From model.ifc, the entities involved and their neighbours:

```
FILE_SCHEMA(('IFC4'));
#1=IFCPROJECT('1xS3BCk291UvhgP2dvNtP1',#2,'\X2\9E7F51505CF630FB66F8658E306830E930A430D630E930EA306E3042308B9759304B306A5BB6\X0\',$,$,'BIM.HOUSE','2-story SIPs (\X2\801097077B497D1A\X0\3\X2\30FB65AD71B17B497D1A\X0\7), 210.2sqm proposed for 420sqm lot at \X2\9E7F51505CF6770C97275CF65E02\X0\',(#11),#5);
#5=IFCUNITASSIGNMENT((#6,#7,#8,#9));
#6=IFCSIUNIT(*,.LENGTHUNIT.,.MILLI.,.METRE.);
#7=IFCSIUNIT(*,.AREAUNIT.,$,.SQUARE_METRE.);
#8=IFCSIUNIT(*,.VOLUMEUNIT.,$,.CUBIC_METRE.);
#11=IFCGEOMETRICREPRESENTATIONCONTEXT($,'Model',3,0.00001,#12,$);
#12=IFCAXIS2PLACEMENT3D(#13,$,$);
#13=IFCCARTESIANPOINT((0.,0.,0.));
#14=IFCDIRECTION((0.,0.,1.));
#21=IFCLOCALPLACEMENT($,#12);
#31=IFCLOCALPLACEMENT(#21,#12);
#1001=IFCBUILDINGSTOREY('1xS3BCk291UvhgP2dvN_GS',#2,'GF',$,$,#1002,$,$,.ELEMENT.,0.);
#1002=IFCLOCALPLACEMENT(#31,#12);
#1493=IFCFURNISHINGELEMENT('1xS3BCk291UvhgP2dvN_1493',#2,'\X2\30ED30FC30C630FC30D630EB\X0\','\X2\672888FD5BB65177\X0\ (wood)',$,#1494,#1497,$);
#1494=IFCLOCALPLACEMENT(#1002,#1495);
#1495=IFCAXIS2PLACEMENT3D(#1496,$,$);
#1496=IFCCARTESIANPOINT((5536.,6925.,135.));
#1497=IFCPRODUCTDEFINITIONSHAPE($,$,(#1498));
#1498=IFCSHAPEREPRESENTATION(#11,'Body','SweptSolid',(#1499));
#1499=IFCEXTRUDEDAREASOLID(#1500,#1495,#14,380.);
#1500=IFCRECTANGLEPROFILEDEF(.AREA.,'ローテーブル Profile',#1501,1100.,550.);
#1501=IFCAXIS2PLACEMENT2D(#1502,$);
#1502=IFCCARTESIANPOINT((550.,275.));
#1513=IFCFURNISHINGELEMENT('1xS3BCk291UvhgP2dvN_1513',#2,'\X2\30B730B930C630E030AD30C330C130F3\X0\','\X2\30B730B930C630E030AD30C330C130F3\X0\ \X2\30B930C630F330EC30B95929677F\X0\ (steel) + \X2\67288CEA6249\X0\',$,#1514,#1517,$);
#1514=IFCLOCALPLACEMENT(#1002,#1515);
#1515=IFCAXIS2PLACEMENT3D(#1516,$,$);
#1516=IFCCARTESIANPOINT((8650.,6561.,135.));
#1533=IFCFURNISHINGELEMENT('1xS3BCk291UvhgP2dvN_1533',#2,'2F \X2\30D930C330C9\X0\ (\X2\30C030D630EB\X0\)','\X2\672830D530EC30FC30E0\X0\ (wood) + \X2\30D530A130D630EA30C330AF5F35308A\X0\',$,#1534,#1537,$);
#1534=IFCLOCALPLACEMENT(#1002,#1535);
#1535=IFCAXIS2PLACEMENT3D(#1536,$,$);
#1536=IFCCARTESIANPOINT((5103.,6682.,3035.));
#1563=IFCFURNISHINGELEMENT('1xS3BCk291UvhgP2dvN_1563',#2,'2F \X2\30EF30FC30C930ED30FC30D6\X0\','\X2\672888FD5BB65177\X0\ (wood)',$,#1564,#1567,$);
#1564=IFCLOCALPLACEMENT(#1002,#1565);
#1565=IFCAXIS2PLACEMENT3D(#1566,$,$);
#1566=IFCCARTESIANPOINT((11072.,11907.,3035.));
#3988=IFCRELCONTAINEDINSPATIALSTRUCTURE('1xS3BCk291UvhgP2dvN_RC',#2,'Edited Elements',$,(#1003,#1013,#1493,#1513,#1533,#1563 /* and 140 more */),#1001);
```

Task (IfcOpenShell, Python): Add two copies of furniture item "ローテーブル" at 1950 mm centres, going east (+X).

```python
import numpy as np
import ifcopenshell
import ifcopenshell.api.geometry
import ifcopenshell.api.root
import ifcopenshell.util.element
import ifcopenshell.util.placement
import ifcopenshell.util.unit

model = ifcopenshell.open("model.ifc")
unit_scale = ifcopenshell.util.unit.calculate_unit_scale(model)


def reuse_history(source, copy):
    """copy_class also copies each property set's owner history, people and application; keep the originals."""
    for rel in copy.IsDefinedBy:
        if rel.is_a("IfcRelDefinesByProperties") and (history := rel.RelatingPropertyDefinition.OwnerHistory):
            rel.RelatingPropertyDefinition.OwnerHistory = source.OwnerHistory
            ifcopenshell.util.element.remove_deep2(model, history)


source = model.by_guid("1xS3BCk291UvhgP2dvN_1493")
base = ifcopenshell.util.placement.get_local_placement(source.ObjectPlacement)
step = np.array([1.0, 0.0, 0.0]) * 1.95 / unit_scale

for i in range(1, 3):
    copy = ifcopenshell.api.root.copy_class(model, product=source)
    copy.Representation = ifcopenshell.util.element.copy_deep(
        model, source.Representation, exclude=["IfcGeometricRepresentationContext", "IfcRepresentationMap"]
    )
    reuse_history(source, copy)
    matrix = base.copy()
    matrix[:3, 3] += i * step
    print("added at", matrix[:3, 3].round(3) + 0.0)
    ifcopenshell.api.geometry.edit_object_placement(model, product=copy, matrix=matrix, is_si=False)

model.write("model_updated.ifc")
```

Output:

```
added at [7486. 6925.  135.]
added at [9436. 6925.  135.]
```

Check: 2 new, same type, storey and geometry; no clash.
